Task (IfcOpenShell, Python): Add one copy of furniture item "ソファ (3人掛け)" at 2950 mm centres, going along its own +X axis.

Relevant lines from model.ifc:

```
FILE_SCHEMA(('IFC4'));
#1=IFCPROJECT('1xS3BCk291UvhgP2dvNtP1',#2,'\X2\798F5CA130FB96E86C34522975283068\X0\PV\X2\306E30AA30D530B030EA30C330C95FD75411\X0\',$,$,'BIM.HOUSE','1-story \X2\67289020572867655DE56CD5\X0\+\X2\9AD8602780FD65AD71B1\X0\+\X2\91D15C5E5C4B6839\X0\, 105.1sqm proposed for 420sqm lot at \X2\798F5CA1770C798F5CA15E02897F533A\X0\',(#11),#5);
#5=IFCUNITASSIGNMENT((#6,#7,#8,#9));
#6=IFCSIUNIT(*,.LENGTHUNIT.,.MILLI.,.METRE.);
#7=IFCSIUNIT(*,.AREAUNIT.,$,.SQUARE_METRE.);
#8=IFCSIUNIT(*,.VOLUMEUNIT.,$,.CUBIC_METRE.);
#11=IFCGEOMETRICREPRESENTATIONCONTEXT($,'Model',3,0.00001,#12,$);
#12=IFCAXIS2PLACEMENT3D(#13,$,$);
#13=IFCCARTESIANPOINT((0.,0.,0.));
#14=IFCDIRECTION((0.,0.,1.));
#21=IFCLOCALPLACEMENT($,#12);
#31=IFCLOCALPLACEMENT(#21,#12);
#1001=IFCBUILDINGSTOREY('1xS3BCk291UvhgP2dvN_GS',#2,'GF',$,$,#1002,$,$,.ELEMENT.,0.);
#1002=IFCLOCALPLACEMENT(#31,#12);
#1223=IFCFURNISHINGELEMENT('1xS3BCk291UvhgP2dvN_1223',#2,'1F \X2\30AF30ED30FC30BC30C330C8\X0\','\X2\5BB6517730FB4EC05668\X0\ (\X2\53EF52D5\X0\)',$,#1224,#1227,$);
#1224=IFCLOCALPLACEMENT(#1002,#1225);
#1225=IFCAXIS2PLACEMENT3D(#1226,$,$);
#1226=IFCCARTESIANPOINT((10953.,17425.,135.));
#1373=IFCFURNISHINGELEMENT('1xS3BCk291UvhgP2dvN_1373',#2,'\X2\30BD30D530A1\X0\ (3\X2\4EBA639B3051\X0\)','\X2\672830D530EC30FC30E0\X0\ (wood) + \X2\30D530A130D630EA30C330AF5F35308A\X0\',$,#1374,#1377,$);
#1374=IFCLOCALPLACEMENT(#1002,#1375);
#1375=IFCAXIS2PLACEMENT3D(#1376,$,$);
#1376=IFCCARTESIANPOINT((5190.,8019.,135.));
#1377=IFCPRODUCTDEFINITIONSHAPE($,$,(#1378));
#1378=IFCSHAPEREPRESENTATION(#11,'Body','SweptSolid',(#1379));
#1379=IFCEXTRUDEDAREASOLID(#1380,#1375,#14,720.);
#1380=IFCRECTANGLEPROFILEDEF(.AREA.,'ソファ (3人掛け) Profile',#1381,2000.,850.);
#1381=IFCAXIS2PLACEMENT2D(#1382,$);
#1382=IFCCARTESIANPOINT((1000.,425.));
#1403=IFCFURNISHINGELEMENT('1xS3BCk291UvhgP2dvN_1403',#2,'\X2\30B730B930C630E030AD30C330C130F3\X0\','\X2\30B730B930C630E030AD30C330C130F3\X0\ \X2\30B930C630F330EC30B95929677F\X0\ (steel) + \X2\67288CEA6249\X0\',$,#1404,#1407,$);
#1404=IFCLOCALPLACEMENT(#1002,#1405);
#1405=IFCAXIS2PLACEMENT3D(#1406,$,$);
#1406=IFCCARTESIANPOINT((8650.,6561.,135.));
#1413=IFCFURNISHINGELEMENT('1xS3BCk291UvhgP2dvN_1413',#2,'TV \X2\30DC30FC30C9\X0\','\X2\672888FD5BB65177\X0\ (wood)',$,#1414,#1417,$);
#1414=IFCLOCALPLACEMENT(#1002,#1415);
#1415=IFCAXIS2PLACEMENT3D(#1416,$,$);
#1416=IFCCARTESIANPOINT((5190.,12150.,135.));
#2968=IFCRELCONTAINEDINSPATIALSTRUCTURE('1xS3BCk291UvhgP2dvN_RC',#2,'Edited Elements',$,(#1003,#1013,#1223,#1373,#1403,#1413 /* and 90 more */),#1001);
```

```python
import ifcopenshell
import ifcopenshell.api.geometry
import ifcopenshell.api.root
import ifcopenshell.util.element
import ifcopenshell.util.placement

model = ifcopenshell.open("model.ifc")


def reuse_history(source, copy):
    """copy_class also copies each property set's owner history, people and application; keep the originals."""
    for rel in copy.IsDefinedBy:
        if rel.is_a("IfcRelDefinesByProperties") and (history := rel.RelatingPropertyDefinition.OwnerHistory):
            rel.RelatingPropertyDefinition.OwnerHistory = source.OwnerHistory
            ifcopenshell.util.element.remove_deep2(model, history)


source = model.by_guid("1xS3BCk291UvhgP2dvN_1373")
base = ifcopenshell.util.placement.get_local_placement(source.ObjectPlacement)
step = base[:3, 0] * 2950.0

for i in range(1, 2):
    copy = ifcopenshell.api.root.copy_class(model, product=source)
    copy.Representation = ifcopenshell.util.element.copy_deep(
        model, source.Representation, exclude=["IfcGeometricRepresentationContext", "IfcRepresentationMap"]
    )
    reuse_history(source, copy)
    matrix = base.copy()
    matrix[:3, 3] += i * step
    print("added at", matrix[:3, 3].round(3) + 0.0)
    ifcopenshell.api.geometry.edit_object_placement(model, product=copy, matrix=matrix, is_si=False)

model.write("model-out.ifc")
```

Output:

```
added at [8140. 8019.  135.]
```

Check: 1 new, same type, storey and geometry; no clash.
